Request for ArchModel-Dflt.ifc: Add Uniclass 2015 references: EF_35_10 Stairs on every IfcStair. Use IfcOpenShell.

First a look at what the model holds.

```python
import ifcopenshell

model = ifcopenshell.open("ArchModel-Dflt.ifc")
print(model.schema)
print("classifications:", [c.Name for c in model.by_type("IfcClassification")])
for ifc_class in ("IfcDoor", "IfcRoof", "IfcStair", "IfcWall", "IfcWindow"):
    print(ifc_class, len(model.by_type(ifc_class)))
```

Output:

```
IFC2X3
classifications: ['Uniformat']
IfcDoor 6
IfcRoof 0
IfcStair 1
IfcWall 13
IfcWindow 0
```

```python
import ifcopenshell
import ifcopenshell.api.classification

model = ifcopenshell.open("ArchModel-Dflt.ifc")

# IFC2X3 requires Source and Edition and has no link from the project to the system.
system = model.create_entity("IfcClassification", Source="NBS", Edition="2015", Name="Uniclass 2015")

codes = {
    "IfcStair": ("EF_35_10", "Stairs"),
}
for ifc_class, (code, name) in codes.items():
    products = model.by_type(ifc_class)
    ifcopenshell.api.classification.add_reference(
        model, products=products, classification=system, identification=code, name=name
    )
    print(code, len(products))

model.write("ArchModel-Dflt_v2.ifc")
```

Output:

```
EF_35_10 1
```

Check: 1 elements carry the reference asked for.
